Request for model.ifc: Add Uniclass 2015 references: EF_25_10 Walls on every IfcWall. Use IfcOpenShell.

First a look at what the model holds.

```python
import ifcopenshell

model = ifcopenshell.open("model.ifc")
print(model.schema)
print("classifications:", [c.Name for c in model.by_type("IfcClassification")])
for ifc_class in ("IfcDoor", "IfcRoof", "IfcStair", "IfcWall", "IfcWindow"):
    print(ifc_class, len(model.by_type(ifc_class)))
```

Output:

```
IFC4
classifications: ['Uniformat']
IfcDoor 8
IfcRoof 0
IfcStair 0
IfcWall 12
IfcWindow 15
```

```python
import ifcopenshell
import ifcopenshell.api.classification

model = ifcopenshell.open("model.ifc")

system = ifcopenshell.api.classification.add_classification(model, classification="Uniclass 2015")

codes = {
    "IfcWall": ("EF_25_10", "Walls"),
}
for ifc_class, (code, name) in codes.items():
    products = model.by_type(ifc_class)
    ifcopenshell.api.classification.add_reference(
        model, products=products, classification=system, identification=code, name=name
    )
    print(code, len(products))

model.write("model_updated.ifc")
```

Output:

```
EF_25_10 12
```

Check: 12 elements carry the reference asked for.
